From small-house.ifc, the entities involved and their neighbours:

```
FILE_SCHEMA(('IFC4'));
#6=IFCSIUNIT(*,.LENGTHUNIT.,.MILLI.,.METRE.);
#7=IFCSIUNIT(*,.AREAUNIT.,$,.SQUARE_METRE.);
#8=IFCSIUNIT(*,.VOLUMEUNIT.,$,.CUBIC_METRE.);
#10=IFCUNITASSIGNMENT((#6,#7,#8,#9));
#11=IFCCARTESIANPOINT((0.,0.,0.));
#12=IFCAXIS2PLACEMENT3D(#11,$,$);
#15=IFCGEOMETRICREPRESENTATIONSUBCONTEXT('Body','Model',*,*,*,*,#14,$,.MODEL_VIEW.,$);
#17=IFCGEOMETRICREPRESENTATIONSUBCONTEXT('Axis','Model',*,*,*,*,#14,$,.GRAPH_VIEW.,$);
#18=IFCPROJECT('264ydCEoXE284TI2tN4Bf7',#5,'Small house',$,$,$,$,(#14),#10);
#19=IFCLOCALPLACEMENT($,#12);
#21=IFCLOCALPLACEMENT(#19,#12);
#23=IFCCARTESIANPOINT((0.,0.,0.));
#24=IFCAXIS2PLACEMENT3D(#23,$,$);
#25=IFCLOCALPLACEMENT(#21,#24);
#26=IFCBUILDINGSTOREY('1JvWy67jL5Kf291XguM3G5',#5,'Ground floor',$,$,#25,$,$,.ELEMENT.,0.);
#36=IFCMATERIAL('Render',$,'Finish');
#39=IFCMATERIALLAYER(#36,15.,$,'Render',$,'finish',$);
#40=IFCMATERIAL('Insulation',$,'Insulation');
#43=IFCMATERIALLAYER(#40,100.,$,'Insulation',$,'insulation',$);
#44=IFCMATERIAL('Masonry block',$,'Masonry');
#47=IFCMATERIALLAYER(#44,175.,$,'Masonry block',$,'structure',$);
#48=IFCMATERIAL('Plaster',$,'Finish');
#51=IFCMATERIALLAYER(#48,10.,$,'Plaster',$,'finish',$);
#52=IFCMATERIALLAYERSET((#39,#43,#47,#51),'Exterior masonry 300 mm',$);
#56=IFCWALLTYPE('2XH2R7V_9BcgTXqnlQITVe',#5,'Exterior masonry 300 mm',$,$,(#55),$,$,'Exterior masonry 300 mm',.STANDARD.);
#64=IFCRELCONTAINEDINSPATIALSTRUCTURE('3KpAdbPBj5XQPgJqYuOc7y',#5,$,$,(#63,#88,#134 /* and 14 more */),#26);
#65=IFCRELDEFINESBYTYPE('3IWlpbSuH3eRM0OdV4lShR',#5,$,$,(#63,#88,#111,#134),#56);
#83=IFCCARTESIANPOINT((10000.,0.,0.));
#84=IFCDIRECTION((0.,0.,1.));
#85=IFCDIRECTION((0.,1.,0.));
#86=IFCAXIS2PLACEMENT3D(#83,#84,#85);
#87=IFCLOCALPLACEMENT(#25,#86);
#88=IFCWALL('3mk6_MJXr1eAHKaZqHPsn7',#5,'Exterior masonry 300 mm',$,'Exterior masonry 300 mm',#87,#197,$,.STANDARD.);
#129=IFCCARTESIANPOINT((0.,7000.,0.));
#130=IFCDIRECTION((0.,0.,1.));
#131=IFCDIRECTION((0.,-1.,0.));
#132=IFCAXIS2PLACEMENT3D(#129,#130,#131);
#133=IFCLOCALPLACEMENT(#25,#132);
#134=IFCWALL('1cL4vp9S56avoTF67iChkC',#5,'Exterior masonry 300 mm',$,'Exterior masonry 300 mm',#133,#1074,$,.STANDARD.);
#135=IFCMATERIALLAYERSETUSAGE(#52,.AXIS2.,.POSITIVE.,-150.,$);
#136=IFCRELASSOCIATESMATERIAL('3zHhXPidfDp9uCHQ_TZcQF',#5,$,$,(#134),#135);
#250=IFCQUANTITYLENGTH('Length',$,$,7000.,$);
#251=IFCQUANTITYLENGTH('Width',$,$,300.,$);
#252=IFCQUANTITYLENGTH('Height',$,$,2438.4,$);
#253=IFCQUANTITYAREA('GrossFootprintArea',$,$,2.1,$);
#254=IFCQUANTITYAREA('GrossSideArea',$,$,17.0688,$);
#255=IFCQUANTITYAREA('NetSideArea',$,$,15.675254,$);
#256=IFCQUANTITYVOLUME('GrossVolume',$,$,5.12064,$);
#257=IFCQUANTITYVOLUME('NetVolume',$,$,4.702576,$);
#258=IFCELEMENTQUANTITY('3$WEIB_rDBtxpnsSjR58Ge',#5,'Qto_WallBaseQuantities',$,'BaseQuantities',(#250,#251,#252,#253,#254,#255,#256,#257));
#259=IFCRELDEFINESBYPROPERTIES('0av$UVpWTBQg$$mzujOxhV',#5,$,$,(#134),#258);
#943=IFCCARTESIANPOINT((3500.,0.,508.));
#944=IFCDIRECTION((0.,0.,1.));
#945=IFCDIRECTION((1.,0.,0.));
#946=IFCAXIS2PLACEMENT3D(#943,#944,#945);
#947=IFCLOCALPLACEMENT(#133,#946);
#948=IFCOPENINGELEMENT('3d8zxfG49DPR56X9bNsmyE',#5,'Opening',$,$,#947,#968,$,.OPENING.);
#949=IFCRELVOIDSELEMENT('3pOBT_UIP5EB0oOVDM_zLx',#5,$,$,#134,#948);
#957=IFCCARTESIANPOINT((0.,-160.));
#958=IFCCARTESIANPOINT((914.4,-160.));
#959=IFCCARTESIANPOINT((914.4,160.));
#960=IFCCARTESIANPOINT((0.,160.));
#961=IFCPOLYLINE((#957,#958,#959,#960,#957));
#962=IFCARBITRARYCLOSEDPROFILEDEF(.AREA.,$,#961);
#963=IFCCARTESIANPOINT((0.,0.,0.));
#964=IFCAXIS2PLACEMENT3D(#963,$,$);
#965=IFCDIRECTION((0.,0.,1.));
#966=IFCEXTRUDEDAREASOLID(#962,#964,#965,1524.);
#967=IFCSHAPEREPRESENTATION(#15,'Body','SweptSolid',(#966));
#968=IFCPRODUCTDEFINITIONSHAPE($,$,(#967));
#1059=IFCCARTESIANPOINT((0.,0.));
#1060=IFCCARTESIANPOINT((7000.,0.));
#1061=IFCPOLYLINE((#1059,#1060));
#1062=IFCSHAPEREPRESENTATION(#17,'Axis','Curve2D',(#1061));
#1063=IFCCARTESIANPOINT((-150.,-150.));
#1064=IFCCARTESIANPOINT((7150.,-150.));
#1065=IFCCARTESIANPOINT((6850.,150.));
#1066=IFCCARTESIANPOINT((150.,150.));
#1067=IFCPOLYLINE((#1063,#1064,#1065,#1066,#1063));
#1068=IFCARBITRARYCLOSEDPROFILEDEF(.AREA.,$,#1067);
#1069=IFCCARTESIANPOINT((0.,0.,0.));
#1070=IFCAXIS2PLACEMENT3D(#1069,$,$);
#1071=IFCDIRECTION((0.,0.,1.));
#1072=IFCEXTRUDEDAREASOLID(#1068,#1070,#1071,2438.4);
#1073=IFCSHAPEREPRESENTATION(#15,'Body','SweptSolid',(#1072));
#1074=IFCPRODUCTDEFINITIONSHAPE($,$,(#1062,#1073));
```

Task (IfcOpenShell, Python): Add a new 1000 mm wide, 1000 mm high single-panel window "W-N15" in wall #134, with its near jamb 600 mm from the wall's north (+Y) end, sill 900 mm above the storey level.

```python
import numpy as np
import ifcopenshell
import ifcopenshell.api.feature
import ifcopenshell.api.geometry
import ifcopenshell.api.pset
import ifcopenshell.api.root
import ifcopenshell.api.spatial
import ifcopenshell.geom
import ifcopenshell.util.element
import ifcopenshell.util.placement
import ifcopenshell.util.representation
import ifcopenshell.util.shape
import ifcopenshell.util.unit

model = ifcopenshell.open("small-house.ifc")
unit_scale = ifcopenshell.util.unit.calculate_unit_scale(model)
area_scale = ifcopenshell.util.unit.calculate_unit_scale(model, "AREAUNIT")
volume_scale = ifcopenshell.util.unit.calculate_unit_scale(model, "VOLUMEUNIT")
settings = ifcopenshell.geom.settings()


def volume(element):
    """Net volume in cubic metres, openings subtracted."""
    shape = ifcopenshell.geom.create_shape(settings, element)
    return ifcopenshell.util.shape.get_volume(shape.geometry)


wall = model.by_guid("1cL4vp9S56avoTF67iChkC")
storey = ifcopenshell.util.element.get_container(wall, ifc_class="IfcBuildingStorey")
context = ifcopenshell.util.representation.get_context(model, "Model", "Body", "MODEL_VIEW")
before = volume(wall)

width, height, from_end, sill = 1, 1, 0.6, 0.9  # metres

# The wall runs along its own X axis, and the end named is its -X end.
wall_shape = ifcopenshell.geom.create_shape(settings, wall)
x, y, z = ifcopenshell.util.shape.get_vertices(wall_shape.geometry).T
start = x.min() + from_end
face, thickness = float(y.min()), float(y.max() - y.min())
wall_matrix = ifcopenshell.util.placement.get_local_placement(wall.ObjectPlacement)
level = ifcopenshell.util.placement.get_local_placement(storey.ObjectPlacement)[2, 3]


def in_wall(x, y):
    """Placement at x, y metres in the wall's axes, at sill height."""
    matrix = wall_matrix.copy()
    matrix[:, 3] = wall_matrix @ np.array([x / unit_scale, y / unit_scale, 0.0, 1.0])
    matrix[2, 3] = level + sill / unit_scale
    return matrix


# Opening: a box that overshoots both wall faces by 50 mm.
opening = ifcopenshell.api.root.create_entity(model, ifc_class="IfcOpeningElement", predefined_type="OPENING")
box = ifcopenshell.api.geometry.add_wall_representation(
    model, context=context, length=width, height=height, thickness=thickness + 0.1
)
ifcopenshell.api.geometry.assign_representation(model, product=opening, representation=box)
ifcopenshell.api.geometry.edit_object_placement(model, product=opening, matrix=in_wall(start, face - 0.05), is_si=False)
ifcopenshell.api.feature.add_feature(model, feature=opening, element=wall)

window = ifcopenshell.api.root.create_entity(model, ifc_class="IfcWindow", name="W-N15", predefined_type="WINDOW")
window.OverallWidth, window.OverallHeight = width / unit_scale, height / unit_scale
window.PartitioningType = "SINGLE_PANEL"
body = ifcopenshell.api.geometry.add_window_representation(
    model,
    context=context,
    overall_width=window.OverallWidth,
    overall_height=window.OverallHeight,
    partition_type="SINGLE_PANEL",
)
ifcopenshell.api.geometry.assign_representation(model, product=window, representation=body)
ifcopenshell.api.spatial.assign_container(model, products=[window], relating_structure=storey)
ifcopenshell.api.feature.add_filling(model, opening=opening, element=window)

# Centre the window in the wall's thickness.
ifcopenshell.api.geometry.edit_object_placement(model, product=window, matrix=in_wall(start, face), is_si=False)
window_shape = ifcopenshell.geom.create_shape(settings, window)
depth = ifcopenshell.util.shape.get_vertices(window_shape.geometry)[:, 1]
offset = face + thickness / 2 - (depth.min() + depth.max()) / 2
ifcopenshell.api.geometry.edit_object_placement(model, product=window, matrix=in_wall(start, offset), is_si=False)

after = volume(wall)

# Update the wall's stored quantities.
qto = model.by_id(ifcopenshell.util.element.get_pset(wall, "Qto_WallBaseQuantities", should_inherit=False)["id"])
ifcopenshell.api.pset.edit_qto(model, qto=qto, properties={
    "NetSideArea": after / thickness / area_scale,
    "NetVolume": after / volume_scale,
})

print(f"wall volume {before:.3f} -> {after:.3f} m3")

model.write("small-house_rev.ifc")
```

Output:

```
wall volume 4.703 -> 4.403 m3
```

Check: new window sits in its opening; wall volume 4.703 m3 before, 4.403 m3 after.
